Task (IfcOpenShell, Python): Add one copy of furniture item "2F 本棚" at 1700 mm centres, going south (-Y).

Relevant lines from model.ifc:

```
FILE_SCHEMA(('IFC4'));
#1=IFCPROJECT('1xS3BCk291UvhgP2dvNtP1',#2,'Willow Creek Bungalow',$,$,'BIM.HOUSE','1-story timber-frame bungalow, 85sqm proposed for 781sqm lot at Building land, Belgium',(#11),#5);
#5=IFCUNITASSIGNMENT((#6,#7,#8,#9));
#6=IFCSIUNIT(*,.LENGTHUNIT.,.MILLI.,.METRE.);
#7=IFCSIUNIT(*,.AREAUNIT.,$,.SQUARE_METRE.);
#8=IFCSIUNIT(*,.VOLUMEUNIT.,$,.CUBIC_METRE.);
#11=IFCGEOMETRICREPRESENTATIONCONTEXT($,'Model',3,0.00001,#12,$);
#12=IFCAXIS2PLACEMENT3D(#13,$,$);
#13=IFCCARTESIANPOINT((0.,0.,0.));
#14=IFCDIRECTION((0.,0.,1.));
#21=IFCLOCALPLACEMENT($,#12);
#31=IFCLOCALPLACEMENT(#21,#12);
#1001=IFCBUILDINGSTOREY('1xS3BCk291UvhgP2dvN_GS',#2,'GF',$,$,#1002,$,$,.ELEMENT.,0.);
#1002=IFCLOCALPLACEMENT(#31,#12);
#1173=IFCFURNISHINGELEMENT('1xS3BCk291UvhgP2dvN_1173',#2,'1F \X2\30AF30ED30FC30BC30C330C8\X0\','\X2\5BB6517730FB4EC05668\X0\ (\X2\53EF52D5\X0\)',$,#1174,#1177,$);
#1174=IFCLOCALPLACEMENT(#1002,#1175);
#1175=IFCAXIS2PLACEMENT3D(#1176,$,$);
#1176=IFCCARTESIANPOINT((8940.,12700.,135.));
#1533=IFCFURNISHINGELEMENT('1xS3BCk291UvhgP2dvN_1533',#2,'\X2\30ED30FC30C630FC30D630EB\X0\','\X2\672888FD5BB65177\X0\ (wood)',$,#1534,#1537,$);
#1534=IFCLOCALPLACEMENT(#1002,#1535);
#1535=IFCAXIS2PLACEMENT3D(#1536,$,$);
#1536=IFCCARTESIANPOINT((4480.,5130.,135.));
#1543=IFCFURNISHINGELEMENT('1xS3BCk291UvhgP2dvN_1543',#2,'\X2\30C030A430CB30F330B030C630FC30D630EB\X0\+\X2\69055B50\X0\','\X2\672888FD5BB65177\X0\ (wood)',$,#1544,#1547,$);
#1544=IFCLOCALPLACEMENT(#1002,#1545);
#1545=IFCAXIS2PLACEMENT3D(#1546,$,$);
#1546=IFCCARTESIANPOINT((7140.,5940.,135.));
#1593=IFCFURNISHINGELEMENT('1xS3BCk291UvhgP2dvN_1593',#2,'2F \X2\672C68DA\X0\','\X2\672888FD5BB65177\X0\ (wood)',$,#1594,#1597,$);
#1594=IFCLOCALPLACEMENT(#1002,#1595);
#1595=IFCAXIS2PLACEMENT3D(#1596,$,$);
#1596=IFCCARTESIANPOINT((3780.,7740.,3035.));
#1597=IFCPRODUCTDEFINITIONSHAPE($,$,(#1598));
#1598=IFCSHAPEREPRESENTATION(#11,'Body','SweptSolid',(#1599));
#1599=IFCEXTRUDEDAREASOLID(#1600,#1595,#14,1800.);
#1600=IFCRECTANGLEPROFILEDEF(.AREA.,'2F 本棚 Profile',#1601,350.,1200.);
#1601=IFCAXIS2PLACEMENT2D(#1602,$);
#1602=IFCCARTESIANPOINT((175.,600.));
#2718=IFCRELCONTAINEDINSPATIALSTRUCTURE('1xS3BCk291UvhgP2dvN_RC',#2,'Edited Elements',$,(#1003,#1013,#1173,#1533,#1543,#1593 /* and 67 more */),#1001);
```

```python
import numpy as np
import ifcopenshell
import ifcopenshell.api.geometry
import ifcopenshell.api.root
import ifcopenshell.util.element
import ifcopenshell.util.placement
import ifcopenshell.util.unit

model = ifcopenshell.open("model.ifc")
unit_scale = ifcopenshell.util.unit.calculate_unit_scale(model)


def reuse_history(source, copy):
    """copy_class also copies each property set's owner history, people and application; keep the originals."""
    for rel in copy.IsDefinedBy:
        if rel.is_a("IfcRelDefinesByProperties") and (history := rel.RelatingPropertyDefinition.OwnerHistory):
            rel.RelatingPropertyDefinition.OwnerHistory = source.OwnerHistory
            ifcopenshell.util.element.remove_deep2(model, history)


source = model.by_guid("1xS3BCk291UvhgP2dvN_1593")
base = ifcopenshell.util.placement.get_local_placement(source.ObjectPlacement)
step = np.array([0.0, -1.0, 0.0]) * 1.7 / unit_scale

for i in range(1, 2):
    copy = ifcopenshell.api.root.copy_class(model, product=source)
    copy.Representation = ifcopenshell.util.element.copy_deep(
        model, source.Representation, exclude=["IfcGeometricRepresentationContext", "IfcRepresentationMap"]
    )
    reuse_history(source, copy)
    matrix = base.copy()
    matrix[:3, 3] += i * step
    print("added at", matrix[:3, 3].round(3) + 0.0)
    ifcopenshell.api.geometry.edit_object_placement(model, product=copy, matrix=matrix, is_si=False)

model.write("model_edited.ifc")
```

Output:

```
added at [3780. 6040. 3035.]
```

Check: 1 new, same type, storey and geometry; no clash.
